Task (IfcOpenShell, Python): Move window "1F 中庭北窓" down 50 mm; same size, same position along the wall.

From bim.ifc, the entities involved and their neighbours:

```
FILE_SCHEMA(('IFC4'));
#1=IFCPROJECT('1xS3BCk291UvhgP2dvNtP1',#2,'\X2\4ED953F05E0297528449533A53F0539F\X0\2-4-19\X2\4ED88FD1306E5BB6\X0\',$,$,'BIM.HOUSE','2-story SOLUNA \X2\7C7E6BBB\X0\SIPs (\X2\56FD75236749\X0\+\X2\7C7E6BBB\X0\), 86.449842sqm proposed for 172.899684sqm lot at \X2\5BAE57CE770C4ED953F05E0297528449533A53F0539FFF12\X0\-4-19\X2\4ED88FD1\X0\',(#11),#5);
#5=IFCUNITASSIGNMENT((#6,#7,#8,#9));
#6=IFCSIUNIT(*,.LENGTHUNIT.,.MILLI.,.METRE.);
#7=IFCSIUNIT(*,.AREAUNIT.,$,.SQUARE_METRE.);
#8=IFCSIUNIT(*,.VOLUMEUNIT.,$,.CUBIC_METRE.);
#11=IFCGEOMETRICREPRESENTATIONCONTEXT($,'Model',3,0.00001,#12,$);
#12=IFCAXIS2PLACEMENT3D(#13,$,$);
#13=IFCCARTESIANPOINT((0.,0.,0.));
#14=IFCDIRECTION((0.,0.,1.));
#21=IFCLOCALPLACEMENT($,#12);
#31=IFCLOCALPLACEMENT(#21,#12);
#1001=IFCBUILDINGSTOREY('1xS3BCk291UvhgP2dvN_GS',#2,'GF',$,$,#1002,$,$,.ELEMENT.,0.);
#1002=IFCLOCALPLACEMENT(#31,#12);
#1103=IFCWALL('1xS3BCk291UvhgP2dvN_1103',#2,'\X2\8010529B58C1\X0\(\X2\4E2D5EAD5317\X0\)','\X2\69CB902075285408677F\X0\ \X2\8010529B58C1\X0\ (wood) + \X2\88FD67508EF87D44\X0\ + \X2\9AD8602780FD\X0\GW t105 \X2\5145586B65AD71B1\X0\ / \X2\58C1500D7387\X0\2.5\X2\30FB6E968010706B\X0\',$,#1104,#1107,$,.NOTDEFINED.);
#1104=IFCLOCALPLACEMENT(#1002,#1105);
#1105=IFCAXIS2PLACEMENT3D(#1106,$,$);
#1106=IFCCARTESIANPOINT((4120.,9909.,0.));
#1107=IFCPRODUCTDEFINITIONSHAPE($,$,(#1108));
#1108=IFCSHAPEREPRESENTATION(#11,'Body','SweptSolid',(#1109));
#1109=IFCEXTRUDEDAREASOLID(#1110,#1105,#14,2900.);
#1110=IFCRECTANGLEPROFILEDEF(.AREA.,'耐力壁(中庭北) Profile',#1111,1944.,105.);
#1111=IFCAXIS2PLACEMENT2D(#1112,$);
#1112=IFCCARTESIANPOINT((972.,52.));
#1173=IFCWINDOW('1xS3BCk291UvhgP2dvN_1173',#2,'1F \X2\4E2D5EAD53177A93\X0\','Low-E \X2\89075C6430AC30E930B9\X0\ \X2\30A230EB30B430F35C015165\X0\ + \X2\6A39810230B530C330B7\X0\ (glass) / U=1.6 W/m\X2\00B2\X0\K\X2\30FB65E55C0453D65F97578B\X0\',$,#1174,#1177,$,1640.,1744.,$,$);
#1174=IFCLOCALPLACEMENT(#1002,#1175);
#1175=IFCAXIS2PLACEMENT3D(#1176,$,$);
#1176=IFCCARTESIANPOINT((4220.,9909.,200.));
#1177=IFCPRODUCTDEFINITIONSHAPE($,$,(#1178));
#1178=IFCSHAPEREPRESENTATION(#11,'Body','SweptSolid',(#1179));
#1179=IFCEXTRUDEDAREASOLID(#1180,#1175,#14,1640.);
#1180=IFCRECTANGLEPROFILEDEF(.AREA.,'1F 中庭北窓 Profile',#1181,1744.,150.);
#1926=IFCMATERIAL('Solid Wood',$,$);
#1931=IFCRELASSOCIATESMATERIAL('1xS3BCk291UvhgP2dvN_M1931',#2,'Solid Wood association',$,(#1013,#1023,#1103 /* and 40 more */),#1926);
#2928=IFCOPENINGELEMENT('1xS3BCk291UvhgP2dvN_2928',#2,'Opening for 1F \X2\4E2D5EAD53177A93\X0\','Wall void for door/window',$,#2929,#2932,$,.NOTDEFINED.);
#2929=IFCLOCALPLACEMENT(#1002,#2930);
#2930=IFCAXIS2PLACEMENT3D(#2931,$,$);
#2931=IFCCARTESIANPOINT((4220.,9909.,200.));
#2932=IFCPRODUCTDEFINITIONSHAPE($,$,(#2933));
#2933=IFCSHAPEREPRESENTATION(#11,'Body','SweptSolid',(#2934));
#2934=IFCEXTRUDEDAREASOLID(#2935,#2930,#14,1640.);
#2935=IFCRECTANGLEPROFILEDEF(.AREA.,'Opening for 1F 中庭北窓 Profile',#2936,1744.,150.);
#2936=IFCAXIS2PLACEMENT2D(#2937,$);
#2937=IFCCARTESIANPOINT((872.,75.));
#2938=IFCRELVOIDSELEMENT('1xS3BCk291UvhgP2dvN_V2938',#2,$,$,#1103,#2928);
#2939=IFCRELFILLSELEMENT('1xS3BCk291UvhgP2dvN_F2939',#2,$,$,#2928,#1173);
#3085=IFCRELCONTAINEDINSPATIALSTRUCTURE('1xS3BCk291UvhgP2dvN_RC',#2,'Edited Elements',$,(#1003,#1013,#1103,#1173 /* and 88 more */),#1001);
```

```python
import numpy as np
import ifcopenshell
import ifcopenshell.api.geometry
import ifcopenshell.util.placement
import ifcopenshell.util.unit

model = ifcopenshell.open("bim.ifc")
unit_scale = ifcopenshell.util.unit.calculate_unit_scale(model)

window = model.by_guid("1xS3BCk291UvhgP2dvN_1173")
opening = window.FillsVoids[0].RelatingOpeningElement
dz = -50.0

shift = np.array([0.0, 0.0, dz])
# The window is not placed relative to its opening, so move both.
for product in (opening, window):
    matrix = ifcopenshell.util.placement.get_local_placement(product.ObjectPlacement)
    matrix[:3, 3] += shift
    ifcopenshell.api.geometry.edit_object_placement(model, product=product, matrix=matrix, is_si=False)

print(f"moved by {dz * unit_scale:+.3f} m")

model.write("bim_v2.ifc")
```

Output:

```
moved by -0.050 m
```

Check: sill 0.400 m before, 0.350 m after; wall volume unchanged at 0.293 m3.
